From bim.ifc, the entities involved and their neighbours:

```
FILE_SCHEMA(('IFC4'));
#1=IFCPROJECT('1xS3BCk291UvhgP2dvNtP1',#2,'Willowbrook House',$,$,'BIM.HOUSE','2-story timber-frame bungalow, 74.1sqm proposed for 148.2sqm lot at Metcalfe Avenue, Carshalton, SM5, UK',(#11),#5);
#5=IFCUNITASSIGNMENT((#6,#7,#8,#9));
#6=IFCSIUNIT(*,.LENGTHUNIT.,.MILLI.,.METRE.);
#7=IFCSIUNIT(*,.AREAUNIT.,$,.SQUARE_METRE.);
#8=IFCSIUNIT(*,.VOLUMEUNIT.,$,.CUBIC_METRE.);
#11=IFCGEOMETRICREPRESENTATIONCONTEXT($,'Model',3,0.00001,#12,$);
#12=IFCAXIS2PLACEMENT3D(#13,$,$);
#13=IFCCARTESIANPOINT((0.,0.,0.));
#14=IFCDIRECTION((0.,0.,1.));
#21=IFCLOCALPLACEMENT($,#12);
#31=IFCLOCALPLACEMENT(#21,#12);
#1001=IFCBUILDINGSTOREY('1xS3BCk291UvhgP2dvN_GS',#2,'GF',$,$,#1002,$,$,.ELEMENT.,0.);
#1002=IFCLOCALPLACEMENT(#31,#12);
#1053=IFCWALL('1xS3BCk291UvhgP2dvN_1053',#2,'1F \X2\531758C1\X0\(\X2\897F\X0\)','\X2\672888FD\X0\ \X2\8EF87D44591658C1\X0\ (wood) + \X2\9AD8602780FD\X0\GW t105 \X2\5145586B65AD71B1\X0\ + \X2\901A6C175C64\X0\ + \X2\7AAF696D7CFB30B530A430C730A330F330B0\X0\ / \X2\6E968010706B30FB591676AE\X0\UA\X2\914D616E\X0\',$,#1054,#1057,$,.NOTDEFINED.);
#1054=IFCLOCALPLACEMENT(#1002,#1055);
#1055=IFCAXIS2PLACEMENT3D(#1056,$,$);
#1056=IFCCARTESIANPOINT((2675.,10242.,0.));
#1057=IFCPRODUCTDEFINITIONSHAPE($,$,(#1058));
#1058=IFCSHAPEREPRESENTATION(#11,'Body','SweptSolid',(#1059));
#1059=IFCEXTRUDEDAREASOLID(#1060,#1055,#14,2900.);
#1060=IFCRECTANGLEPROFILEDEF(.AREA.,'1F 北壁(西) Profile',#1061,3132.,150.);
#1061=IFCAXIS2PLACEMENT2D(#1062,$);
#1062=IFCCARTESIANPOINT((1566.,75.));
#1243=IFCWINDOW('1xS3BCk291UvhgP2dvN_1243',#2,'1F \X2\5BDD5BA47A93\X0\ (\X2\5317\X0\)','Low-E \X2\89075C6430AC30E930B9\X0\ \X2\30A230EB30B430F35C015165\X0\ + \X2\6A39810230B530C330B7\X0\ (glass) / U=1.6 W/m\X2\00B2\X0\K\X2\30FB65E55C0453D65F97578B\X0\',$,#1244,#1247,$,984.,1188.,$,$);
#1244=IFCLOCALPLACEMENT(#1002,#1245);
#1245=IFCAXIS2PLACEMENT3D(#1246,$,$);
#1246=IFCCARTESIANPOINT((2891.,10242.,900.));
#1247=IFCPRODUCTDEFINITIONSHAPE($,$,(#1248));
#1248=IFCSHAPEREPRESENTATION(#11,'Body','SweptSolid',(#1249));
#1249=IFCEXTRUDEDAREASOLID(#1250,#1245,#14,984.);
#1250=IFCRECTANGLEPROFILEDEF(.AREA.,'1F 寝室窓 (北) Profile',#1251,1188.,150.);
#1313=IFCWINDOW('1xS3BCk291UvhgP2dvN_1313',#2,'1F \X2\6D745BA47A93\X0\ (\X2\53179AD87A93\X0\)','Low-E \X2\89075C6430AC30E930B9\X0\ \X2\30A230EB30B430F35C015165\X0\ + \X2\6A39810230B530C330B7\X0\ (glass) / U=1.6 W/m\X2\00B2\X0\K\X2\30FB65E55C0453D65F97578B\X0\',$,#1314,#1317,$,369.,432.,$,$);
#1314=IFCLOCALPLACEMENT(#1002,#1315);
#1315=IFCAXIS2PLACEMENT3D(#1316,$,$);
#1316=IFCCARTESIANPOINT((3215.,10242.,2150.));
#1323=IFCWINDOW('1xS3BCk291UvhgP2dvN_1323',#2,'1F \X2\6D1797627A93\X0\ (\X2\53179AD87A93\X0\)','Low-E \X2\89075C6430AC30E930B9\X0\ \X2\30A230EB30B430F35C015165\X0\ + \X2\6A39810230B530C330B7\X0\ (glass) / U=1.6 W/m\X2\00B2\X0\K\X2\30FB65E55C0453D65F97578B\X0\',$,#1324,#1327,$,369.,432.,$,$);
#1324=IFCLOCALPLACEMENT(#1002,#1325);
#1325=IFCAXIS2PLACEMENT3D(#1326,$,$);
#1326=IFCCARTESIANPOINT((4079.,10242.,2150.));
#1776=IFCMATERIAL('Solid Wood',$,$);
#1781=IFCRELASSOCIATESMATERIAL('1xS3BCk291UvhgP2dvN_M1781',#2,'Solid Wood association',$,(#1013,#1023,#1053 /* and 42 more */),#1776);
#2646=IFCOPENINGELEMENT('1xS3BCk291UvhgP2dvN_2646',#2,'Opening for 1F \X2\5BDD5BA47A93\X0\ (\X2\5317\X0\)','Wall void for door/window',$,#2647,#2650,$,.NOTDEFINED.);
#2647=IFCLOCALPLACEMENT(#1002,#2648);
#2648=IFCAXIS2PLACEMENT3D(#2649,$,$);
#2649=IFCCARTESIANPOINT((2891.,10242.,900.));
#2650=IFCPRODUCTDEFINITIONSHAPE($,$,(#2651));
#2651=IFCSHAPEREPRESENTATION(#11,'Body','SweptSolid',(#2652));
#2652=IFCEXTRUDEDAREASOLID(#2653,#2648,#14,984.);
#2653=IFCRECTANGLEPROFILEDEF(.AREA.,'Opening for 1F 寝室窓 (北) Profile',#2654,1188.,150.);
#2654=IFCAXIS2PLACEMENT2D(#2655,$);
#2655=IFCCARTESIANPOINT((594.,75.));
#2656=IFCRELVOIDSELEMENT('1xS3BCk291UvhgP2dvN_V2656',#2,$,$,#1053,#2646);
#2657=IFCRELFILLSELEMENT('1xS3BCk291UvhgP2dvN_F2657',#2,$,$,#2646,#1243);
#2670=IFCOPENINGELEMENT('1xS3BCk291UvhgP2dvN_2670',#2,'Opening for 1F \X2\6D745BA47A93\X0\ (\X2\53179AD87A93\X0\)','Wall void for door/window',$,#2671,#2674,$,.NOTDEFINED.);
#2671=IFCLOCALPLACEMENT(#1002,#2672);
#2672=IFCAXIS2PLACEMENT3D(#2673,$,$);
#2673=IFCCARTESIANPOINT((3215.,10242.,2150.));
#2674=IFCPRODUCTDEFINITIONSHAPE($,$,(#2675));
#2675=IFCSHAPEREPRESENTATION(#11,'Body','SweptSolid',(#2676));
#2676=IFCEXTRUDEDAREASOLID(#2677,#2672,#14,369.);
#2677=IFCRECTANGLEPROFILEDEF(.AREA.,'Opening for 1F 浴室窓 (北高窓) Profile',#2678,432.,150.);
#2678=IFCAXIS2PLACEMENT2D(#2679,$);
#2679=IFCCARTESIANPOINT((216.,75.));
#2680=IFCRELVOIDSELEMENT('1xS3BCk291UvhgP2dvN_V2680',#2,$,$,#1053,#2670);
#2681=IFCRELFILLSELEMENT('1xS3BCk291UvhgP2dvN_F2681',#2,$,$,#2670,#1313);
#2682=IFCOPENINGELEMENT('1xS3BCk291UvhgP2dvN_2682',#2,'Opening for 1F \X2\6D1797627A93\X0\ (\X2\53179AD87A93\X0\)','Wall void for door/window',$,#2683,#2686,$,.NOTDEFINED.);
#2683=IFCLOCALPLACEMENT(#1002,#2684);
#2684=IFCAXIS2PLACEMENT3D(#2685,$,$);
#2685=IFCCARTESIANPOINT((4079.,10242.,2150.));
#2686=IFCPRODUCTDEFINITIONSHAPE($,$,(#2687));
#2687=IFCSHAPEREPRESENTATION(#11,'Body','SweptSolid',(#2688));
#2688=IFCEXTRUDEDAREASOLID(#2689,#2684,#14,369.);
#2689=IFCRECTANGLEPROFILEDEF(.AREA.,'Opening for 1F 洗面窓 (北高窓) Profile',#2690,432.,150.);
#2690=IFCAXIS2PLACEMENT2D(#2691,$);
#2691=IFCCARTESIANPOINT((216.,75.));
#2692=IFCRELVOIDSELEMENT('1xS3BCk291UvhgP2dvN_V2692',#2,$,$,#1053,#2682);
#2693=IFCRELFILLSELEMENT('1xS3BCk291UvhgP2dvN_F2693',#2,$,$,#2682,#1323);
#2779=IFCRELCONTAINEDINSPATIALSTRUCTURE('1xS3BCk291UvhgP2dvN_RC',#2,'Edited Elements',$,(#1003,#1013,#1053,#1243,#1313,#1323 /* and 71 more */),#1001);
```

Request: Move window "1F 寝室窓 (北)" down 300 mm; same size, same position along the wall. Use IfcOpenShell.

```python
import numpy as np
import ifcopenshell
import ifcopenshell.api.geometry
import ifcopenshell.util.placement
import ifcopenshell.util.unit

model = ifcopenshell.open("bim.ifc")
unit_scale = ifcopenshell.util.unit.calculate_unit_scale(model)

window = model.by_guid("1xS3BCk291UvhgP2dvN_1243")
opening = window.FillsVoids[0].RelatingOpeningElement
dz = -0.3 / unit_scale

shift = np.array([0.0, 0.0, dz])
# The window is not placed relative to its opening, so move both.
for product in (opening, window):
    matrix = ifcopenshell.util.placement.get_local_placement(product.ObjectPlacement)
    matrix[:3, 3] += shift
    ifcopenshell.api.geometry.edit_object_placement(model, product=product, matrix=matrix, is_si=False)

print(f"moved by {dz * unit_scale:+.3f} m")

model.write("bim_rev.ifc")
```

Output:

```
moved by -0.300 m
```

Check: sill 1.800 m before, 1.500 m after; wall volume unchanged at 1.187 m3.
